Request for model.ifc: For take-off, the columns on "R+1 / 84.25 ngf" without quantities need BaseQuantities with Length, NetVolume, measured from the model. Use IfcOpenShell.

First a look at what the model holds.

```python
import ifcopenshell
import ifcopenshell.util.element
import ifcopenshell.util.unit

model = ifcopenshell.open("model.ifc")
print(model.schema)
for unit_type in ("LENGTHUNIT", "AREAUNIT", "VOLUMEUNIT"):
    print(unit_type, ifcopenshell.util.unit.calculate_unit_scale(model, unit_type))
storey = next(s for s in model.by_type("IfcBuildingStorey") if s.Name == "R+1 / 84.25 ngf")
columns = [e for e in ifcopenshell.util.element.get_decomposition(storey) if e.is_a("IfcColumn")]
for e in sorted(columns, key=lambda e: e.id()):
    print(e.id(), e.is_a(), e.Name, list(ifcopenshell.util.element.get_psets(e, qtos_only=True)), sep=" | ")
```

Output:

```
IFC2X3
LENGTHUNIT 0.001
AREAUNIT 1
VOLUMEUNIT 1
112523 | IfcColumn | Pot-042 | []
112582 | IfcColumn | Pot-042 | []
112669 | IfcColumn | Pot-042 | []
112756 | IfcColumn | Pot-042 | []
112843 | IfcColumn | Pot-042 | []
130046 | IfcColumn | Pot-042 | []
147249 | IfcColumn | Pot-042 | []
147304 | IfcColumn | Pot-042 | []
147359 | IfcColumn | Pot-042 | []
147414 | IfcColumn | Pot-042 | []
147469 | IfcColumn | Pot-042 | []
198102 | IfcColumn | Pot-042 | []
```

```python
import ifcopenshell
import ifcopenshell.api.pset
import ifcopenshell.geom
import ifcopenshell.util.element
import ifcopenshell.util.shape
import ifcopenshell.util.unit

model = ifcopenshell.open("model.ifc")
unit_scale = ifcopenshell.util.unit.calculate_unit_scale(model)
volume_scale = ifcopenshell.util.unit.calculate_unit_scale(model, "VOLUMEUNIT")
settings = ifcopenshell.geom.settings()

storey = next(s for s in model.by_type("IfcBuildingStorey") if s.Name == "R+1 / 84.25 ngf")
columns = [e for e in ifcopenshell.util.element.get_decomposition(storey) if e.is_a("IfcColumn")]

for e in sorted(columns, key=lambda e: e.id()):
    if ifcopenshell.util.element.get_psets(e, qtos_only=True, should_inherit=False):
        continue
    # Geometry comes back in metres, in the element's own axes.
    shape = ifcopenshell.geom.create_shape(settings, e)
    values = {
        "Length": ifcopenshell.util.shape.get_z(shape.geometry) / unit_scale,
        "NetVolume": ifcopenshell.util.shape.get_volume(shape.geometry) / volume_scale,
    }
    qto = ifcopenshell.api.pset.add_qto(model, product=e, name="BaseQuantities")
    ifcopenshell.api.pset.edit_qto(model, qto=qto, properties=values)
    print(e.id(), {k: round(v, 3) for k, v in values.items()})

model.write("model-out.ifc")
```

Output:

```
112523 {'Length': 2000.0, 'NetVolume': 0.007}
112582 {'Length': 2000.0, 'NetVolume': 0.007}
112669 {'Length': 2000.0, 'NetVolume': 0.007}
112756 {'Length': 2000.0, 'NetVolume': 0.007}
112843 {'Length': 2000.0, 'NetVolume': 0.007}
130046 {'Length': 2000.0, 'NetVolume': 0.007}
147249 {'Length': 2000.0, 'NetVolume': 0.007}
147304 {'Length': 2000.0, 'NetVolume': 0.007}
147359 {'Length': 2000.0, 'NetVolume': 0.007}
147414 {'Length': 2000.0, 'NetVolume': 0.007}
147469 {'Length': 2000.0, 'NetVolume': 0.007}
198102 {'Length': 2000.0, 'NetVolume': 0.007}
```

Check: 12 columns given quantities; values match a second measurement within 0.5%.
